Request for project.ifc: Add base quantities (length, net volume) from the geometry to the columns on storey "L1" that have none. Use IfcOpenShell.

First a look at what the model holds.

```python
import ifcopenshell
import ifcopenshell.util.element
import ifcopenshell.util.unit

model = ifcopenshell.open("project.ifc")
print(model.schema)
for unit_type in ("LENGTHUNIT", "AREAUNIT", "VOLUMEUNIT"):
    print(unit_type, ifcopenshell.util.unit.calculate_unit_scale(model, unit_type))
storey = next(s for s in model.by_type("IfcBuildingStorey") if s.Name == "L1")
columns = [e for e in ifcopenshell.util.element.get_decomposition(storey) if e.is_a("IfcColumn")]
for e in sorted(columns, key=lambda e: e.id()):
    print(e.id(), e.is_a(), e.Name, list(ifcopenshell.util.element.get_psets(e, qtos_only=True)), sep=" | ")
```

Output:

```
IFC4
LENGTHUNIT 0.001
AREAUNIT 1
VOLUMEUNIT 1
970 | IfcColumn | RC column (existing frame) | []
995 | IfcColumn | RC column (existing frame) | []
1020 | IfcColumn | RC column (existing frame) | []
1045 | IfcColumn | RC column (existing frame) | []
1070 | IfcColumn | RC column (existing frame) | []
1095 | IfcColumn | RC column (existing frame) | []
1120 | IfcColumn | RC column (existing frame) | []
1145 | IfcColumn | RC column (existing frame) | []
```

```python
import ifcopenshell
import ifcopenshell.api.pset
import ifcopenshell.geom
import ifcopenshell.util.element
import ifcopenshell.util.shape
import ifcopenshell.util.unit

model = ifcopenshell.open("project.ifc")
unit_scale = ifcopenshell.util.unit.calculate_unit_scale(model)
volume_scale = ifcopenshell.util.unit.calculate_unit_scale(model, "VOLUMEUNIT")
settings = ifcopenshell.geom.settings()

storey = next(s for s in model.by_type("IfcBuildingStorey") if s.Name == "L1")
columns = [e for e in ifcopenshell.util.element.get_decomposition(storey) if e.is_a("IfcColumn")]

for e in sorted(columns, key=lambda e: e.id()):
    if ifcopenshell.util.element.get_psets(e, qtos_only=True, should_inherit=False):
        continue
    # Geometry comes back in metres, in the element's own axes.
    shape = ifcopenshell.geom.create_shape(settings, e)
    values = {
        "Length": ifcopenshell.util.shape.get_z(shape.geometry) / unit_scale,
        "NetVolume": ifcopenshell.util.shape.get_volume(shape.geometry) / volume_scale,
    }
    qto = ifcopenshell.api.pset.add_qto(model, product=e, name="Qto_ColumnBaseQuantities")
    ifcopenshell.api.pset.edit_qto(model, qto=qto, properties=values)
    print(e.id(), {k: round(v, 3) for k, v in values.items()})

model.write("project_rev.ifc")
```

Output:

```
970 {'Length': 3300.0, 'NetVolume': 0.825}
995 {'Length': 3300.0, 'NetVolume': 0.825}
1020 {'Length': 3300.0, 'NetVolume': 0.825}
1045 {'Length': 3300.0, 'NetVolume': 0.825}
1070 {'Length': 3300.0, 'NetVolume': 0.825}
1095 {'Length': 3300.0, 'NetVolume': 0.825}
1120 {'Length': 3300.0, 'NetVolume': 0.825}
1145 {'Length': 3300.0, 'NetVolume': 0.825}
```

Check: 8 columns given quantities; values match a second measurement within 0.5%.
